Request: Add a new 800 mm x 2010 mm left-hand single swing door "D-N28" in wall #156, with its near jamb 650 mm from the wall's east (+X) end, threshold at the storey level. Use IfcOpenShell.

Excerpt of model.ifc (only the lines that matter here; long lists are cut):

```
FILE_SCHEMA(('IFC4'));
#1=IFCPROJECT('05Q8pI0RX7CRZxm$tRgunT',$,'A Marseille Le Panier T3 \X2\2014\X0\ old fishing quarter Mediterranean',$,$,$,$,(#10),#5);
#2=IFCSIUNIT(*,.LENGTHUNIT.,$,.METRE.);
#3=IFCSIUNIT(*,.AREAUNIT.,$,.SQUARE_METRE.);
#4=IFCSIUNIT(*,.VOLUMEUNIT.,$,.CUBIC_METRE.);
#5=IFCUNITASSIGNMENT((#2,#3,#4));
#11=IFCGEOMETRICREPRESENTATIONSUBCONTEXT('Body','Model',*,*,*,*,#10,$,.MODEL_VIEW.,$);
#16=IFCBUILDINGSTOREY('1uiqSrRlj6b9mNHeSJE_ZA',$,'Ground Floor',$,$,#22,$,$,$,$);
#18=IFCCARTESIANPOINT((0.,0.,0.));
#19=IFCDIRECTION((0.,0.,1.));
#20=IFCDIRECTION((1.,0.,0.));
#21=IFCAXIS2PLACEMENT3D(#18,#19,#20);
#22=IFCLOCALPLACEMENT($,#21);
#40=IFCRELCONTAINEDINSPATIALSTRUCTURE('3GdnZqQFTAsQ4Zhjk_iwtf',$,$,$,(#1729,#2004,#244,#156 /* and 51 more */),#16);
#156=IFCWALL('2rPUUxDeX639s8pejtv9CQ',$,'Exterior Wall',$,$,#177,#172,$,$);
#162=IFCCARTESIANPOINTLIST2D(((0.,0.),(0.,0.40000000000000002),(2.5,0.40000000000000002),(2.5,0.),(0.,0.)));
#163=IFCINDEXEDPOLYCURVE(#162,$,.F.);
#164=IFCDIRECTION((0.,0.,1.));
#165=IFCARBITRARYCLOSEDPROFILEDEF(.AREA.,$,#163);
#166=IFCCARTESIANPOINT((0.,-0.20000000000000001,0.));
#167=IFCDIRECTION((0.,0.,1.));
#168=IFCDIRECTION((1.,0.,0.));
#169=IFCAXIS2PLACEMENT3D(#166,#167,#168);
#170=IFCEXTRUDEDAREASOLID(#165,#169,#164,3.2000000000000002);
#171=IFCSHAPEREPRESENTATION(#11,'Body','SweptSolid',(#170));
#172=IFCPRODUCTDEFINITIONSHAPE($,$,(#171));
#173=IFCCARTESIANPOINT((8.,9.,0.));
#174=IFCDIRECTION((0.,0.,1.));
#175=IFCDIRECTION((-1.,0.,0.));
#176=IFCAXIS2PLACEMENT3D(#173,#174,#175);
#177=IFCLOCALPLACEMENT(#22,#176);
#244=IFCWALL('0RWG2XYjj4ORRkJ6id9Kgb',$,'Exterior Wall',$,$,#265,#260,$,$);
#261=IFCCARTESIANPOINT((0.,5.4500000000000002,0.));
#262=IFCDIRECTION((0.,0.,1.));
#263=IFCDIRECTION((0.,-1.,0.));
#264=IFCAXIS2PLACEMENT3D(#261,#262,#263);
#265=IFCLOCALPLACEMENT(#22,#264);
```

```python
import numpy as np
import ifcopenshell
import ifcopenshell.api.feature
import ifcopenshell.api.geometry
import ifcopenshell.api.root
import ifcopenshell.api.spatial
import ifcopenshell.geom
import ifcopenshell.util.element
import ifcopenshell.util.placement
import ifcopenshell.util.representation
import ifcopenshell.util.shape
import ifcopenshell.util.unit

model = ifcopenshell.open("model.ifc")
unit_scale = ifcopenshell.util.unit.calculate_unit_scale(model)
settings = ifcopenshell.geom.settings()


def volume(element):
    """Net volume in cubic metres, openings subtracted."""
    shape = ifcopenshell.geom.create_shape(settings, element)
    return ifcopenshell.util.shape.get_volume(shape.geometry)


wall = model.by_guid("2rPUUxDeX639s8pejtv9CQ")
storey = ifcopenshell.util.element.get_container(wall, ifc_class="IfcBuildingStorey")
context = ifcopenshell.util.representation.get_context(model, "Model", "Body", "MODEL_VIEW")
before = volume(wall)

width, height, from_end, sill = 0.8, 2.01, 0.65, 0.0  # metres

# The wall runs along its own X axis, and the end named is its -X end.
wall_shape = ifcopenshell.geom.create_shape(settings, wall)
x, y, z = ifcopenshell.util.shape.get_vertices(wall_shape.geometry).T
start = x.min() + from_end
face, thickness = float(y.min()), float(y.max() - y.min())
wall_matrix = ifcopenshell.util.placement.get_local_placement(wall.ObjectPlacement)
level = ifcopenshell.util.placement.get_local_placement(storey.ObjectPlacement)[2, 3]


def in_wall(x, y):
    """Placement at x, y metres in the wall's axes, at sill height."""
    matrix = wall_matrix.copy()
    matrix[:, 3] = wall_matrix @ np.array([x / unit_scale, y / unit_scale, 0.0, 1.0])
    matrix[2, 3] = level + sill / unit_scale
    return matrix


# Opening: a box that overshoots both wall faces by 50 mm.
opening = ifcopenshell.api.root.create_entity(model, ifc_class="IfcOpeningElement", predefined_type="OPENING")
box = ifcopenshell.api.geometry.add_wall_representation(
    model, context=context, length=width, height=height, thickness=thickness + 0.1
)
ifcopenshell.api.geometry.assign_representation(model, product=opening, representation=box)
ifcopenshell.api.geometry.edit_object_placement(model, product=opening, matrix=in_wall(start, face - 0.05), is_si=False)
ifcopenshell.api.feature.add_feature(model, feature=opening, element=wall)

door = ifcopenshell.api.root.create_entity(model, ifc_class="IfcDoor", name="D-N28", predefined_type="DOOR")
door.OverallWidth, door.OverallHeight = width / unit_scale, height / unit_scale
door.OperationType = "SINGLE_SWING_LEFT"
body = ifcopenshell.api.geometry.add_door_representation(
    model,
    context=context,
    overall_width=door.OverallWidth,
    overall_height=door.OverallHeight,
    operation_type="SINGLE_SWING_LEFT",
    lining_properties={"LiningDepth": thickness / unit_scale, "ThresholdDepth": thickness / unit_scale},
)
ifcopenshell.api.geometry.assign_representation(model, product=door, representation=body)
ifcopenshell.api.spatial.assign_container(model, products=[door], relating_structure=storey)
ifcopenshell.api.feature.add_filling(model, opening=opening, element=door)

# The lining spans the wall, so the door starts at the wall face.
ifcopenshell.api.geometry.edit_object_placement(model, product=door, matrix=in_wall(start, face), is_si=False)

after = volume(wall)

print(f"wall volume {before:.3f} -> {after:.3f} m3")

model.write("model-out.ifc")
```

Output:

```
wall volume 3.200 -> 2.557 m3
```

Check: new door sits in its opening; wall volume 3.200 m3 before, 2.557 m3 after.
